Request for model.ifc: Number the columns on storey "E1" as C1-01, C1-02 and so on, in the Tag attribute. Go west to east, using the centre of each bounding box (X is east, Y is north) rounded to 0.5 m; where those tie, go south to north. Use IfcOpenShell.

First a look at what the model holds.

```python
import ifcopenshell
import ifcopenshell.util.element
import ifcopenshell.util.placement

model = ifcopenshell.open("model.ifc")
print(model.schema)
storey = next(s for s in model.by_type("IfcBuildingStorey") if s.Name == "E1")
columns = [e for e in ifcopenshell.util.element.get_decomposition(storey) if e.is_a("IfcColumn")]
for e in sorted(columns, key=lambda e: e.id()):
    origin = ifcopenshell.util.placement.get_local_placement(e.ObjectPlacement)[:3, 3]
    print(e.id(), e.Tag, e.Name, origin.round(2) + 0.0, sep=" | ")
```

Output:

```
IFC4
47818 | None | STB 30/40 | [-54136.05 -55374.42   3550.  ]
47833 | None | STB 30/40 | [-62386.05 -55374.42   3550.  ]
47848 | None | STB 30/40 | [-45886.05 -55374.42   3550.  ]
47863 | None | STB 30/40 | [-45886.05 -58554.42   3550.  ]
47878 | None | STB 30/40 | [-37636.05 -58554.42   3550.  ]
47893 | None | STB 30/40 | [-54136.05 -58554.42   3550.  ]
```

```python
import ifcopenshell
import ifcopenshell.geom
import ifcopenshell.util.element
import ifcopenshell.util.shape

model = ifcopenshell.open("model.ifc")
settings = ifcopenshell.geom.settings()
settings.set("use-world-coords", True)


def centre(element):
    shape = ifcopenshell.geom.create_shape(settings, element)
    return ifcopenshell.util.shape.get_bbox_centroid(shape.geometry)


storey = next(s for s in model.by_type("IfcBuildingStorey") if s.Name == "E1")
columns = [e for e in ifcopenshell.util.element.get_decomposition(storey) if e.is_a("IfcColumn")]

# Insertion points can sit at a corner or the storey origin, so sort by the geometry (in metres).
centres = {e: centre(e) for e in columns}
columns.sort(key=lambda e: (round(centres[e][0] / 0.5), centres[e][1]))

for i, e in enumerate(columns, start=1):
    number = f"C1-{i:02d}"
    e.Tag = number
    print(e.id(), number)

model.write("model_edited.ifc")
```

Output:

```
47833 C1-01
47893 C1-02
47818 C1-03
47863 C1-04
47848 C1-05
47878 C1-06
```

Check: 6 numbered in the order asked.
